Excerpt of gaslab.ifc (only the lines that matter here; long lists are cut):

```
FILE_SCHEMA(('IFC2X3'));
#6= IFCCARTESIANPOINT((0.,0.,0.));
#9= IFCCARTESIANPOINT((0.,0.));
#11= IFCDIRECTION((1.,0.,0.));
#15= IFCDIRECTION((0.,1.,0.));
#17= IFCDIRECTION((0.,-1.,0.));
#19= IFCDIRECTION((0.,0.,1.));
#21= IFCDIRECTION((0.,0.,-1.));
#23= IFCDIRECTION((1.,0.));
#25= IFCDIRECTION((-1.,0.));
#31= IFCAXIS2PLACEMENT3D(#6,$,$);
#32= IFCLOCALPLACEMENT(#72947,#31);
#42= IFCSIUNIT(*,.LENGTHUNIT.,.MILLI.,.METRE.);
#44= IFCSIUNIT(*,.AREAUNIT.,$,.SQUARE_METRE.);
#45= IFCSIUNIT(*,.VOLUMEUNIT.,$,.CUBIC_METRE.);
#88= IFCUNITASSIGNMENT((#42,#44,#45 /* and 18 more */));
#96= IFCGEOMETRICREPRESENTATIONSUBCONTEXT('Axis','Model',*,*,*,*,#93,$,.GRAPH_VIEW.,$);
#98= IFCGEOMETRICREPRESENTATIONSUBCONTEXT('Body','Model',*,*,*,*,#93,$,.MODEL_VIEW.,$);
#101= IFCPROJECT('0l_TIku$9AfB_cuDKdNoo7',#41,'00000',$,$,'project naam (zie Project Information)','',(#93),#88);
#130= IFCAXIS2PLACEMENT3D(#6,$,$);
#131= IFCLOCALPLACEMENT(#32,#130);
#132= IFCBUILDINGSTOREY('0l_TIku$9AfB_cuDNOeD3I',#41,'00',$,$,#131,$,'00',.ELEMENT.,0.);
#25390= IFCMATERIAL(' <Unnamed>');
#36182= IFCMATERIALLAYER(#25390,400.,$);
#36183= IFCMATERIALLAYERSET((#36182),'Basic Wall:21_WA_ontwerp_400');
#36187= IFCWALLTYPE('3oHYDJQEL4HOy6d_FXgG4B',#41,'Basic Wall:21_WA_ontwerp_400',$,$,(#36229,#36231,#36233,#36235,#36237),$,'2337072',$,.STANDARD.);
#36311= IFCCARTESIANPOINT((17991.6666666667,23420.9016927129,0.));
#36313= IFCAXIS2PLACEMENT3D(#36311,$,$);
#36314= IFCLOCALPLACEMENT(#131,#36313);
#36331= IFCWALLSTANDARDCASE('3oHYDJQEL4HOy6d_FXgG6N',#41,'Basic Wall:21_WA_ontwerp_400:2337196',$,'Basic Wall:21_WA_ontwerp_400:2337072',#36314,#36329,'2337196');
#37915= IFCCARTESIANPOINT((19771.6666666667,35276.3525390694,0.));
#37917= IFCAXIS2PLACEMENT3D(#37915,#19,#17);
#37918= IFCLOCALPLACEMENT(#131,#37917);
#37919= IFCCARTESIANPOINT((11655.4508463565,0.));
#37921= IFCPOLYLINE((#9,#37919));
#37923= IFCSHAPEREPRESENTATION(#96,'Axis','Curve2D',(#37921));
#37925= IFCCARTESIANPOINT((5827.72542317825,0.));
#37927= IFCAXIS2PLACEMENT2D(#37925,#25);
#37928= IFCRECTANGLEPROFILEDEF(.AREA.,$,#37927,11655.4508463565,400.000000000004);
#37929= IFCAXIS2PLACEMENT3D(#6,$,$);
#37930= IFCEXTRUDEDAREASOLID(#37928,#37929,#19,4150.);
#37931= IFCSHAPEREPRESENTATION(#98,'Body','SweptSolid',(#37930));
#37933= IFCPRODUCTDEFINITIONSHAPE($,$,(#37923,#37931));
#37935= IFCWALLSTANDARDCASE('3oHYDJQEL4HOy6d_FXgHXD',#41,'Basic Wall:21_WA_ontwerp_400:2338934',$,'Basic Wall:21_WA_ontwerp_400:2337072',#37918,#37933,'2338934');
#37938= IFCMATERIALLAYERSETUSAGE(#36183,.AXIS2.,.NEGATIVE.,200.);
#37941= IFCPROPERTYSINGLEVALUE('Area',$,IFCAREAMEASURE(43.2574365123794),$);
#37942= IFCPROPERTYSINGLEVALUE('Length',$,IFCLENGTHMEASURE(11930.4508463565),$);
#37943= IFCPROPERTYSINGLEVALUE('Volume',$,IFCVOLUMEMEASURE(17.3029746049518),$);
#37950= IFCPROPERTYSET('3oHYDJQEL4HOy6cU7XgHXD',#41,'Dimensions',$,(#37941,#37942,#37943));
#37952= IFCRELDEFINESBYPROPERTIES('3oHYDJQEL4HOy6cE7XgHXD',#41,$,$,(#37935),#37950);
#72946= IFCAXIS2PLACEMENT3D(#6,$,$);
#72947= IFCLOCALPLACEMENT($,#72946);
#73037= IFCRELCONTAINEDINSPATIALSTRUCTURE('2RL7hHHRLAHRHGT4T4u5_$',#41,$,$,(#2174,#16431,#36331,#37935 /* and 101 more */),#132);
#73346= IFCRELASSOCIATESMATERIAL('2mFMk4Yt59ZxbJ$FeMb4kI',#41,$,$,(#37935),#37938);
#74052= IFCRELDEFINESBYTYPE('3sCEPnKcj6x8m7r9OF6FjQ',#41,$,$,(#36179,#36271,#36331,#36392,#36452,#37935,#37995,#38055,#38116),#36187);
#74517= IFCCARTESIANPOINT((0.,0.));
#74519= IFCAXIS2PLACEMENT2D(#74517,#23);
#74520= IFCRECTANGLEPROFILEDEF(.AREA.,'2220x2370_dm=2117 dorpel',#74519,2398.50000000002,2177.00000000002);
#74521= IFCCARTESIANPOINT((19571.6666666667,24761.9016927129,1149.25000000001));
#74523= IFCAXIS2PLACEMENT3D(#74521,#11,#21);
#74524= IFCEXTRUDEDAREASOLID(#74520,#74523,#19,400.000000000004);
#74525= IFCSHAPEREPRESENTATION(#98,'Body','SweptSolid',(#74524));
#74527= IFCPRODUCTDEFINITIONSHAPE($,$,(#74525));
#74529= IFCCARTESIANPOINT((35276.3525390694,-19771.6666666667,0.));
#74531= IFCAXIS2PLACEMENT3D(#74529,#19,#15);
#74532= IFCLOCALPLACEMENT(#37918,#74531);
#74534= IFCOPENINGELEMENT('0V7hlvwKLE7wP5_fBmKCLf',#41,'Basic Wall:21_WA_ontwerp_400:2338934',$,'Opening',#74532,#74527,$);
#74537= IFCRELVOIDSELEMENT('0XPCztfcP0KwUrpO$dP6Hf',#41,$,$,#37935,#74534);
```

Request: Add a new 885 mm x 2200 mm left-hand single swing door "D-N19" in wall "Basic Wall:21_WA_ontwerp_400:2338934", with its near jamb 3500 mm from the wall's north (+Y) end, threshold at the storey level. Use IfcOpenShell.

```python
import numpy as np
import ifcopenshell
import ifcopenshell.api.feature
import ifcopenshell.api.geometry
import ifcopenshell.api.pset
import ifcopenshell.api.root
import ifcopenshell.api.spatial
import ifcopenshell.api.type
import ifcopenshell.geom
import ifcopenshell.util.element
import ifcopenshell.util.placement
import ifcopenshell.util.representation
import ifcopenshell.util.shape
import ifcopenshell.util.unit

model = ifcopenshell.open("gaslab.ifc")
unit_scale = ifcopenshell.util.unit.calculate_unit_scale(model)
area_scale = ifcopenshell.util.unit.calculate_unit_scale(model, "AREAUNIT")
volume_scale = ifcopenshell.util.unit.calculate_unit_scale(model, "VOLUMEUNIT")
settings = ifcopenshell.geom.settings()


def volume(element):
    """Net volume in cubic metres, openings subtracted."""
    shape = ifcopenshell.geom.create_shape(settings, element)
    return ifcopenshell.util.shape.get_volume(shape.geometry)


wall = model.by_id(37935)
storey = ifcopenshell.util.element.get_container(wall, ifc_class="IfcBuildingStorey")
context = ifcopenshell.util.representation.get_context(model, "Model", "Body", "MODEL_VIEW")
before = volume(wall)

width, height, from_end, sill = 0.885, 2.2, 3.5, 0.0  # metres

# The wall runs along its own X axis, and the end named is its -X end.
wall_shape = ifcopenshell.geom.create_shape(settings, wall)
x, y, z = ifcopenshell.util.shape.get_vertices(wall_shape.geometry).T
start = x.min() + from_end
face, thickness = float(y.min()), float(y.max() - y.min())
wall_matrix = ifcopenshell.util.placement.get_local_placement(wall.ObjectPlacement)
level = ifcopenshell.util.placement.get_local_placement(storey.ObjectPlacement)[2, 3]


def in_wall(x, y):
    """Placement at x, y metres in the wall's axes, at sill height."""
    matrix = wall_matrix.copy()
    matrix[:, 3] = wall_matrix @ np.array([x / unit_scale, y / unit_scale, 0.0, 1.0])
    matrix[2, 3] = level + sill / unit_scale
    return matrix


# Opening: a box that overshoots both wall faces by 50 mm.
opening = ifcopenshell.api.root.create_entity(model, ifc_class="IfcOpeningElement")
box = ifcopenshell.api.geometry.add_wall_representation(
    model, context=context, length=width, height=height, thickness=thickness + 0.1
)
ifcopenshell.api.geometry.assign_representation(model, product=opening, representation=box)
ifcopenshell.api.geometry.edit_object_placement(model, product=opening, matrix=in_wall(start, face - 0.05), is_si=False)
ifcopenshell.api.feature.add_feature(model, feature=opening, element=wall)

door = ifcopenshell.api.root.create_entity(model, ifc_class="IfcDoor", name="D-N19")
door.OverallWidth, door.OverallHeight = width / unit_scale, height / unit_scale
body = ifcopenshell.api.geometry.add_door_representation(
    model,
    context=context,
    overall_width=door.OverallWidth,
    overall_height=door.OverallHeight,
    operation_type="SINGLE_SWING_LEFT",
    lining_properties={"LiningDepth": thickness / unit_scale, "ThresholdDepth": thickness / unit_scale},
)
ifcopenshell.api.geometry.assign_representation(model, product=door, representation=body)
ifcopenshell.api.spatial.assign_container(model, products=[door], relating_structure=storey)
fills = ifcopenshell.api.feature.add_filling(model, opening=opening, element=door)
fills.OwnerHistory = door.OwnerHistory  # required in IFC2X3

# IFC2X3 keeps the operation on the door style.
style = ifcopenshell.api.root.create_entity(model, ifc_class="IfcDoorStyle", name="D-N19")
style.OperationType, style.ConstructionType = "SINGLE_SWING_LEFT", "NOTDEFINED"
style.ParameterTakesPrecedence = style.Sizeable = False
ifcopenshell.api.type.assign_type(model, related_objects=[door], relating_type=style)

# The lining spans the wall, so the door starts at the wall face.
ifcopenshell.api.geometry.edit_object_placement(model, product=door, matrix=in_wall(start, face), is_si=False)

after = volume(wall)

# Update the wall's stored quantities.
pset = model.by_id(ifcopenshell.util.element.get_pset(wall, "Dimensions", should_inherit=False)["id"])
ifcopenshell.api.pset.edit_pset(model, pset=pset, properties={
    "Area": model.create_entity("IfcAreaMeasure", after / thickness / area_scale),
    "Volume": model.create_entity("IfcVolumeMeasure", after / volume_scale),
})

print(f"wall volume {before:.3f} -> {after:.3f} m3")

model.write("gaslab_edited.ifc")
```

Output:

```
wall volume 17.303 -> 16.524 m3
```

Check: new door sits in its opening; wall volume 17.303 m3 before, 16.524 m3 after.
